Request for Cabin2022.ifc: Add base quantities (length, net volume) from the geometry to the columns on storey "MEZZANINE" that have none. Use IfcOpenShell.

First a look at what the model holds.

```python
import ifcopenshell
import ifcopenshell.util.element
import ifcopenshell.util.unit

model = ifcopenshell.open("Cabin2022.ifc")
print(model.schema)
for unit_type in ("LENGTHUNIT", "AREAUNIT", "VOLUMEUNIT"):
    print(unit_type, ifcopenshell.util.unit.calculate_unit_scale(model, unit_type))
storey = next(s for s in model.by_type("IfcBuildingStorey") if s.Name == "MEZZANINE")
columns = [e for e in ifcopenshell.util.element.get_decomposition(storey) if e.is_a("IfcColumn")]
for e in sorted(columns, key=lambda e: e.id()):
    print(e.id(), e.is_a(), e.Name, list(ifcopenshell.util.element.get_psets(e, qtos_only=True)), sep=" | ")
```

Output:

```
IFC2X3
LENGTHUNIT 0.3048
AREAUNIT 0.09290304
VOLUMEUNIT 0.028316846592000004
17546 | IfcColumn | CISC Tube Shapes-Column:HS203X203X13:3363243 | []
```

```python
import ifcopenshell
import ifcopenshell.api.pset
import ifcopenshell.geom
import ifcopenshell.util.element
import ifcopenshell.util.shape
import ifcopenshell.util.unit

model = ifcopenshell.open("Cabin2022.ifc")
unit_scale = ifcopenshell.util.unit.calculate_unit_scale(model)
volume_scale = ifcopenshell.util.unit.calculate_unit_scale(model, "VOLUMEUNIT")
settings = ifcopenshell.geom.settings()

storey = next(s for s in model.by_type("IfcBuildingStorey") if s.Name == "MEZZANINE")
columns = [e for e in ifcopenshell.util.element.get_decomposition(storey) if e.is_a("IfcColumn")]

for e in sorted(columns, key=lambda e: e.id()):
    if ifcopenshell.util.element.get_psets(e, qtos_only=True, should_inherit=False):
        continue
    # Geometry comes back in metres, in the element's own axes.
    shape = ifcopenshell.geom.create_shape(settings, e)
    values = {
        "Length": ifcopenshell.util.shape.get_z(shape.geometry) / unit_scale,
        "NetVolume": ifcopenshell.util.shape.get_volume(shape.geometry) / volume_scale,
    }
    qto = ifcopenshell.api.pset.add_qto(model, product=e, name="BaseQuantities")
    ifcopenshell.api.pset.edit_qto(model, qto=qto, properties=values)
    print(e.id(), {k: round(v, 3) for k, v in values.items()})

model.write("Cabin2022_updated.ifc")
```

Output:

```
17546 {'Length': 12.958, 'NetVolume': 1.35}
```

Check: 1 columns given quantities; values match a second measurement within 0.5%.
